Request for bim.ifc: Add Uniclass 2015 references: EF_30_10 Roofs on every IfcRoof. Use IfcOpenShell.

First a look at what the model holds.

```python
import ifcopenshell

model = ifcopenshell.open("bim.ifc")
print(model.schema)
print("classifications:", [c.Name for c in model.by_type("IfcClassification")])
for ifc_class in ("IfcDoor", "IfcRoof", "IfcStair", "IfcWall", "IfcWindow"):
    print(ifc_class, len(model.by_type(ifc_class)))
```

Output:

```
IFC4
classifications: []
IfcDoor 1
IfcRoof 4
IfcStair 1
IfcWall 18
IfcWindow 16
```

```python
import ifcopenshell
import ifcopenshell.api.classification

model = ifcopenshell.open("bim.ifc")

system = ifcopenshell.api.classification.add_classification(model, classification="Uniclass 2015")

codes = {
    "IfcRoof": ("EF_30_10", "Roofs"),
}
for ifc_class, (code, name) in codes.items():
    products = model.by_type(ifc_class)
    ifcopenshell.api.classification.add_reference(
        model, products=products, classification=system, identification=code, name=name
    )
    print(code, len(products))

model.write("bim_rev.ifc")
```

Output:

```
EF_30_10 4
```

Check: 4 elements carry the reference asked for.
